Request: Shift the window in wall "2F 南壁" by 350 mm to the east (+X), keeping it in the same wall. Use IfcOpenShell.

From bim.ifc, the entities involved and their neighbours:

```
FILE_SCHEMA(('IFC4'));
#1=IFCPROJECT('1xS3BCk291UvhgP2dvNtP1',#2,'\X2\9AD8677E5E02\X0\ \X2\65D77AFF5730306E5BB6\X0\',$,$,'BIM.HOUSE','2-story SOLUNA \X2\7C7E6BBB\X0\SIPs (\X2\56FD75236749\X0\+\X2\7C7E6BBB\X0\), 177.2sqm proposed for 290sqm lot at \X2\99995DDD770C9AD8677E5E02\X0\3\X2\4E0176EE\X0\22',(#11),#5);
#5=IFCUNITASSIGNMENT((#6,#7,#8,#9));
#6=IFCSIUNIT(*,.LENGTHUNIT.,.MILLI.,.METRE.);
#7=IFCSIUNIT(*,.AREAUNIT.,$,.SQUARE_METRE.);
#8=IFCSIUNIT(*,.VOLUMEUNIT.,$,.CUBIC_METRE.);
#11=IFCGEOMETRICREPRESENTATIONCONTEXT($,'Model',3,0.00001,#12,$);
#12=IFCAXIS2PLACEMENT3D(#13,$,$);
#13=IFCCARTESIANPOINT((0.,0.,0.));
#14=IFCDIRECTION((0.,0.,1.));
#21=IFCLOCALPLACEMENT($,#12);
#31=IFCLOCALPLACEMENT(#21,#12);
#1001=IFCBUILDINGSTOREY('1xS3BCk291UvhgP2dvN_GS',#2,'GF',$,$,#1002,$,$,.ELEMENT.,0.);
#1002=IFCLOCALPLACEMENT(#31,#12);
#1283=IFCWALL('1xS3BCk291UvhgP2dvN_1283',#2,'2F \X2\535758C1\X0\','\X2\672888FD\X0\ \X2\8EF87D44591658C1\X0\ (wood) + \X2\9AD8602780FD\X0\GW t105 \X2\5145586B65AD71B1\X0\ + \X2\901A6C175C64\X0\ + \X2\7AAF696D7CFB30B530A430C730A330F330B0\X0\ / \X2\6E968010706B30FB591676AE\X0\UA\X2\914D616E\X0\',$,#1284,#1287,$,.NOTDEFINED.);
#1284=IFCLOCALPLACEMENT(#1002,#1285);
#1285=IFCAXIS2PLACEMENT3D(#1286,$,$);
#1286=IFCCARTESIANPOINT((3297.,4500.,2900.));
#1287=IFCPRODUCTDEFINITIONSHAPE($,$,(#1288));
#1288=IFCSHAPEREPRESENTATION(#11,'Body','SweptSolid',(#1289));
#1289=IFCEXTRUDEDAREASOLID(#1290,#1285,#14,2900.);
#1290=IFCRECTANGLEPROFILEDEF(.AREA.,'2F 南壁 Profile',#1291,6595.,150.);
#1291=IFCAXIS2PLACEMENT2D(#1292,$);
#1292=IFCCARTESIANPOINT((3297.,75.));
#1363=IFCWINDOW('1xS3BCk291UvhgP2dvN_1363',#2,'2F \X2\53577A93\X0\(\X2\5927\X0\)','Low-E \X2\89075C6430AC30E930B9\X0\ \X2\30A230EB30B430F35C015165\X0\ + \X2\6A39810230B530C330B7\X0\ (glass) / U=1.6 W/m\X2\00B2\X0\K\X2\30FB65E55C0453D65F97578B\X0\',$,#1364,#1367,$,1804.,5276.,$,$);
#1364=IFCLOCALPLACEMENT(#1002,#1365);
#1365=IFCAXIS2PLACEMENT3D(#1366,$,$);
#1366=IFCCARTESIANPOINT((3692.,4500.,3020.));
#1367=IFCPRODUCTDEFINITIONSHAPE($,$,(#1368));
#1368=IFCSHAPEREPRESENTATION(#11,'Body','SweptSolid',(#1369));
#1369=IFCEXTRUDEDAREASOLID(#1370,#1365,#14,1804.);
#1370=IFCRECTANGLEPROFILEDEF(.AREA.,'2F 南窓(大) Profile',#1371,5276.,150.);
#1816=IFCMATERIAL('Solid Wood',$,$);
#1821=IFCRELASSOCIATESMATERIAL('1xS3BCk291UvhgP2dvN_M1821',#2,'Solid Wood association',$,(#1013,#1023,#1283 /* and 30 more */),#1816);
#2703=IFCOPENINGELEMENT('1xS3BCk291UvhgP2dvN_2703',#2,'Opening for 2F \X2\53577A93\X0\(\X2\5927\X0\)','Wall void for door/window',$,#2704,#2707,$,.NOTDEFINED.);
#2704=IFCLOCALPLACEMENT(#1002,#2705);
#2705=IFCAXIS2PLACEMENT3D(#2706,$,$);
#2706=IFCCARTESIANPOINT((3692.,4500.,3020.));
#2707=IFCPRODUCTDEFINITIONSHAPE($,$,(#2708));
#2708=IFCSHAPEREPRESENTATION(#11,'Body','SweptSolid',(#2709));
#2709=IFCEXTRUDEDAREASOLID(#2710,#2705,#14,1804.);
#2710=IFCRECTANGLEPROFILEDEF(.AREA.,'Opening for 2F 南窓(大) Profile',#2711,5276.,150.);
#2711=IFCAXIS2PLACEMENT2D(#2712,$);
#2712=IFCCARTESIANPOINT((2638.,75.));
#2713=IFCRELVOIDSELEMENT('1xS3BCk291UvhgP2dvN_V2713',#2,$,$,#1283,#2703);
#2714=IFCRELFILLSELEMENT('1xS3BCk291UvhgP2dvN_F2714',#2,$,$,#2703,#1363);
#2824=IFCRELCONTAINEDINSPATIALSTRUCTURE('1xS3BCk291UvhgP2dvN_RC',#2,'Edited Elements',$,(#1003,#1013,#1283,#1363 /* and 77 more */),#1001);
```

```python
import ifcopenshell
import ifcopenshell.api.geometry
import ifcopenshell.util.placement

model = ifcopenshell.open("bim.ifc")

window = model.by_guid("1xS3BCk291UvhgP2dvN_1363")
opening = window.FillsVoids[0].RelatingOpeningElement
wall = opening.VoidsElements[0].RelatingBuildingElement

wall_matrix = ifcopenshell.util.placement.get_local_placement(wall.ObjectPlacement)
shift = wall_matrix[:3, 0] * 350.0
before = ifcopenshell.util.placement.get_local_placement(window.ObjectPlacement)[:3, 3].copy()

# The window is not placed relative to its opening, so move both.
for product in (opening, window):
    matrix = ifcopenshell.util.placement.get_local_placement(product.ObjectPlacement)
    matrix[:3, 3] += shift
    ifcopenshell.api.geometry.edit_object_placement(model, product=product, matrix=matrix, is_si=False)

after = ifcopenshell.util.placement.get_local_placement(window.ObjectPlacement)[:3, 3]
print("window moved by", (after - before).round(3) + 0.0)

model.write("bim_v2.ifc")
```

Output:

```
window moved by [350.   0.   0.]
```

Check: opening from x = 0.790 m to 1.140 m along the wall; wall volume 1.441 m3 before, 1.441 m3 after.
